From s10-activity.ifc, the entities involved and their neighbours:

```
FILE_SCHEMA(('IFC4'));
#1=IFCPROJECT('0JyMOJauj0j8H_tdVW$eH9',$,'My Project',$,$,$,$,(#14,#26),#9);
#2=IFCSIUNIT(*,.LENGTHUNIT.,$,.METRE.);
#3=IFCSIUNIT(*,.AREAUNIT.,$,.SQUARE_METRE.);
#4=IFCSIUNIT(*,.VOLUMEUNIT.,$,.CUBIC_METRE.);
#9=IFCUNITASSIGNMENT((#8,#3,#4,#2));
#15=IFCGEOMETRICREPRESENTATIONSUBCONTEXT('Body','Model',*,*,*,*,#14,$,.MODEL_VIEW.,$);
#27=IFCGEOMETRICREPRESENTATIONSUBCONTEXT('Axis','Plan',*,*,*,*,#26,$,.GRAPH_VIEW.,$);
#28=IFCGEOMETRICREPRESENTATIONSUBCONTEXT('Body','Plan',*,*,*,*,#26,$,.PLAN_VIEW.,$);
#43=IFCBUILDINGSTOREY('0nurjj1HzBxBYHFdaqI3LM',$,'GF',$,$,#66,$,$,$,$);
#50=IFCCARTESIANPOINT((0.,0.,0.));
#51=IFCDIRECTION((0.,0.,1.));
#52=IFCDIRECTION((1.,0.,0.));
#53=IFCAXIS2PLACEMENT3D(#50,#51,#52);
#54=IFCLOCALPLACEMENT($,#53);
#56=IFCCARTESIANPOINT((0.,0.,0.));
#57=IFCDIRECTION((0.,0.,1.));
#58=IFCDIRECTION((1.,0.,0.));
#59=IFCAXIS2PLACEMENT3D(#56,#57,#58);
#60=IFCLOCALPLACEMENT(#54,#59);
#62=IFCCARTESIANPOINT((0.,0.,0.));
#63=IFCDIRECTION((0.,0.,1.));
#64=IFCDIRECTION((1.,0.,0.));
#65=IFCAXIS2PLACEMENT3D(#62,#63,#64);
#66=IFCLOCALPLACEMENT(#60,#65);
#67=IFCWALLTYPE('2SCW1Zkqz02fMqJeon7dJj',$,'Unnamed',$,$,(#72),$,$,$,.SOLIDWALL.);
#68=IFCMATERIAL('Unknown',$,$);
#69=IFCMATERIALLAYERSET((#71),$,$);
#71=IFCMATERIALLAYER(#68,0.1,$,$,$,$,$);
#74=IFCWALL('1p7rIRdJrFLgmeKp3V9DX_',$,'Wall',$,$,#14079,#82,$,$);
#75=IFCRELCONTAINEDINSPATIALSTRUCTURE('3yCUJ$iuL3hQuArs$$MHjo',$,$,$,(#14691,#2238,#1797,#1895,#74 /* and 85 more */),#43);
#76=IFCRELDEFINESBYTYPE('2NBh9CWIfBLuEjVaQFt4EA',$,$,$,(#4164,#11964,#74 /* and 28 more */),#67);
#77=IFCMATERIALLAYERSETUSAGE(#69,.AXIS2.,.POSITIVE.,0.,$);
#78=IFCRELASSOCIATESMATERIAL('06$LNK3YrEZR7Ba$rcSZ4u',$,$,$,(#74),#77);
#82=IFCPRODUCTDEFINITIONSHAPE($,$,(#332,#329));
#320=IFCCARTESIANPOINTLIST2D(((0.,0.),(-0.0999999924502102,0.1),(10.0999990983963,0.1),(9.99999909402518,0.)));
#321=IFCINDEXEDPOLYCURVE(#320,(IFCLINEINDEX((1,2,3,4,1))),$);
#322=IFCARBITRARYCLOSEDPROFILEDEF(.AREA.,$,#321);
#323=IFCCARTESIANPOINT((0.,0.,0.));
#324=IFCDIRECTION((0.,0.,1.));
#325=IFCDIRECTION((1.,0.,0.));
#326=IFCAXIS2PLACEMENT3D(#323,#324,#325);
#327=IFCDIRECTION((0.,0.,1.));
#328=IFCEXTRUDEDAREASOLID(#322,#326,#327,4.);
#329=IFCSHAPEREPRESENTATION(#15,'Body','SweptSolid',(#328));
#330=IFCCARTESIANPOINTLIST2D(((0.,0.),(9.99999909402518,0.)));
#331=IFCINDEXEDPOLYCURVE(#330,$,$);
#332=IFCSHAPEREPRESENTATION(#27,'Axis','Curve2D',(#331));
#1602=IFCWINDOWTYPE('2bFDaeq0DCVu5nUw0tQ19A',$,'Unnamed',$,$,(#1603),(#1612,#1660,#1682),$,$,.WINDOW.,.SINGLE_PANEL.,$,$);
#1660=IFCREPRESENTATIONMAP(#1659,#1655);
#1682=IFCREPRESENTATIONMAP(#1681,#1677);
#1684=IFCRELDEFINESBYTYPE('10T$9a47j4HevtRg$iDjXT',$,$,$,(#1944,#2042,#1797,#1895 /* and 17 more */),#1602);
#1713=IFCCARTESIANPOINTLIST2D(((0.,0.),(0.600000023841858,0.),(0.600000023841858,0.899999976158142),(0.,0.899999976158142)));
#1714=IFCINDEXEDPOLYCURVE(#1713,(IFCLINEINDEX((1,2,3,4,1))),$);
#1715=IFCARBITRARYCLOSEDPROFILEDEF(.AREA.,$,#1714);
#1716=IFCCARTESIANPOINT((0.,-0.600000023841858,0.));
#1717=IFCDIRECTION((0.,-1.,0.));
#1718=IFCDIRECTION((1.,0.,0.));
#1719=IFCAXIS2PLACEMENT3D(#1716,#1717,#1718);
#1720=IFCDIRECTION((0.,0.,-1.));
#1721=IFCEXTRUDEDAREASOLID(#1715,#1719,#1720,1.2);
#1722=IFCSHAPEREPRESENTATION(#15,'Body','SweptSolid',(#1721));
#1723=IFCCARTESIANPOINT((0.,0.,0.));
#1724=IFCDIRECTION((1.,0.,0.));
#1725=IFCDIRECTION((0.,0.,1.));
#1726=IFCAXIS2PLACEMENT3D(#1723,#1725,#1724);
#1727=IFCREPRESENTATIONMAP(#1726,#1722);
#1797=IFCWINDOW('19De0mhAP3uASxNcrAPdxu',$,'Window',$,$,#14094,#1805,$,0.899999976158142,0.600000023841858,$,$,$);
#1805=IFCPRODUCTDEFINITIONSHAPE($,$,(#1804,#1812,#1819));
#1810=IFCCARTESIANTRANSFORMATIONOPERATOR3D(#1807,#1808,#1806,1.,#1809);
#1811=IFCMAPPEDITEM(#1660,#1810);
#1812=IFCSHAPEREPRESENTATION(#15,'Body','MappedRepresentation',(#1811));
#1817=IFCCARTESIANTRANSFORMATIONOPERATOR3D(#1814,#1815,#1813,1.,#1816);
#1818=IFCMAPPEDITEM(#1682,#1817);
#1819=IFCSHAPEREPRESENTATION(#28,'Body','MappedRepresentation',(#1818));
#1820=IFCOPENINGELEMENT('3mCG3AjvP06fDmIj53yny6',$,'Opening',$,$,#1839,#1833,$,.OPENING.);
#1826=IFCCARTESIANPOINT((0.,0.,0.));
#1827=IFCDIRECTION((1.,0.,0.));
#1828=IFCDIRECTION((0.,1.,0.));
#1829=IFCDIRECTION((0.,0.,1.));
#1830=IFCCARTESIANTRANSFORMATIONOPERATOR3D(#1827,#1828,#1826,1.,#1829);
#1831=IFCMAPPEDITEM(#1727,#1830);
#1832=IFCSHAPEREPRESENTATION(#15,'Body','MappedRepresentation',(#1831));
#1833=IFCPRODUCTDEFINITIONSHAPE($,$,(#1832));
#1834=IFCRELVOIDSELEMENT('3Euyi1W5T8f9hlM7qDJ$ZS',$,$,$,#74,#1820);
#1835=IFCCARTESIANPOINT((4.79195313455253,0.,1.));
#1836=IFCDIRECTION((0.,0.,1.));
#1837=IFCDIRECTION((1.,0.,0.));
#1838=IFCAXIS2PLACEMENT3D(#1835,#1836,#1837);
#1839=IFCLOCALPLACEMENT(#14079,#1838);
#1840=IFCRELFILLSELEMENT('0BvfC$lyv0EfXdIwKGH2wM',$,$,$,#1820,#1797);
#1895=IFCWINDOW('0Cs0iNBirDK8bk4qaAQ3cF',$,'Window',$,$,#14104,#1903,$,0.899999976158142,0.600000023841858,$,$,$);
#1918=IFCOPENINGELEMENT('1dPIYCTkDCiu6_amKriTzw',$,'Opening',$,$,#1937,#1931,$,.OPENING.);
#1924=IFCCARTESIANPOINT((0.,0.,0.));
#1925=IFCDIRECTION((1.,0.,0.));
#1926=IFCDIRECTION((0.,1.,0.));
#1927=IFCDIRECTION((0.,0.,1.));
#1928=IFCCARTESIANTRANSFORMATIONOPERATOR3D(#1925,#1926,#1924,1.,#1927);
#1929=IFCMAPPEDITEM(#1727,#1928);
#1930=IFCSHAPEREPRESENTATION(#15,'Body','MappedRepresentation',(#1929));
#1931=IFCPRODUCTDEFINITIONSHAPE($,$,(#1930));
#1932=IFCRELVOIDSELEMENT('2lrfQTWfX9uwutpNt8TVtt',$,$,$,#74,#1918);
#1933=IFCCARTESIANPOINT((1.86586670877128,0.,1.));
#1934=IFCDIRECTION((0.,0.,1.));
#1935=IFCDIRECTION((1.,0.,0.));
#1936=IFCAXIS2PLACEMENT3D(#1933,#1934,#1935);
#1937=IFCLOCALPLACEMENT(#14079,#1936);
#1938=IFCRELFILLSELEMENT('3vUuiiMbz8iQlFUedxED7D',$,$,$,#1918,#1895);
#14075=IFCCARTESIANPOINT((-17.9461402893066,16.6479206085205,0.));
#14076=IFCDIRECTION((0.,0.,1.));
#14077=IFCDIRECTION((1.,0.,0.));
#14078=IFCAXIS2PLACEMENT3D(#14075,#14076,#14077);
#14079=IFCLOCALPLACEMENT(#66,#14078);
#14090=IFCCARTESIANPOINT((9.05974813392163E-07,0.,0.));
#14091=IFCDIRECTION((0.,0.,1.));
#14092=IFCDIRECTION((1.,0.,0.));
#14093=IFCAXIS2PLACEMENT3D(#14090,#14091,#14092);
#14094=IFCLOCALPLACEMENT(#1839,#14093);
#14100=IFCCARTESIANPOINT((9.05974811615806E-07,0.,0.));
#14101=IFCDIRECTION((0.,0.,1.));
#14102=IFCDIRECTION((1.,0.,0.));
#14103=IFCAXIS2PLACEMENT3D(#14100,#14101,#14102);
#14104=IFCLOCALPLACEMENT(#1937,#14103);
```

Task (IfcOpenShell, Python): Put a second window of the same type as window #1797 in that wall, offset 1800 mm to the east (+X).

```python
import ifcopenshell
import ifcopenshell.api.feature
import ifcopenshell.api.geometry
import ifcopenshell.api.root
import ifcopenshell.geom
import ifcopenshell.util.element
import ifcopenshell.util.placement
import ifcopenshell.util.shape
import ifcopenshell.util.unit

model = ifcopenshell.open("s10-activity.ifc")
unit_scale = ifcopenshell.util.unit.calculate_unit_scale(model)
settings = ifcopenshell.geom.settings()


def volume(element):
    """Net volume in cubic metres, openings subtracted."""
    shape = ifcopenshell.geom.create_shape(settings, element)
    return ifcopenshell.util.shape.get_volume(shape.geometry)


window = model.by_guid("19De0mhAP3uASxNcrAPdxu")
opening = window.FillsVoids[0].RelatingOpeningElement
wall = opening.VoidsElements[0].RelatingBuildingElement
before = volume(wall)
shift = ifcopenshell.util.placement.get_local_placement(wall.ObjectPlacement)[:3, 0] * 1.8 / unit_scale

# copy_class copies the void relationship, type, container and properties, but no geometry.
new_opening = ifcopenshell.api.root.copy_class(model, product=opening)
new_opening.Representation = ifcopenshell.util.element.copy_deep(
    model, opening.Representation, exclude=["IfcGeometricRepresentationContext", "IfcRepresentationMap"]
)
new_window = ifcopenshell.api.root.copy_class(model, product=window)
new_window.Representation = ifcopenshell.util.element.copy_deep(
    model, window.Representation, exclude=["IfcGeometricRepresentationContext", "IfcRepresentationMap"]
)
ifcopenshell.api.feature.add_filling(model, opening=new_opening, element=new_window)

for old, new in ((opening, new_opening), (window, new_window)):
    matrix = ifcopenshell.util.placement.get_local_placement(old.ObjectPlacement)
    matrix[:3, 3] += shift
    ifcopenshell.api.geometry.edit_object_placement(model, product=new, matrix=matrix, is_si=False)

after = volume(wall)

print(f"wall volume {before:.3f} -> {after:.3f} m3")

model.write("s10-activity_rev.ifc")
```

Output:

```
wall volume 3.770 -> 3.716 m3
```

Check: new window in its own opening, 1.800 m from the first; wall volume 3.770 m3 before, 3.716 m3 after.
